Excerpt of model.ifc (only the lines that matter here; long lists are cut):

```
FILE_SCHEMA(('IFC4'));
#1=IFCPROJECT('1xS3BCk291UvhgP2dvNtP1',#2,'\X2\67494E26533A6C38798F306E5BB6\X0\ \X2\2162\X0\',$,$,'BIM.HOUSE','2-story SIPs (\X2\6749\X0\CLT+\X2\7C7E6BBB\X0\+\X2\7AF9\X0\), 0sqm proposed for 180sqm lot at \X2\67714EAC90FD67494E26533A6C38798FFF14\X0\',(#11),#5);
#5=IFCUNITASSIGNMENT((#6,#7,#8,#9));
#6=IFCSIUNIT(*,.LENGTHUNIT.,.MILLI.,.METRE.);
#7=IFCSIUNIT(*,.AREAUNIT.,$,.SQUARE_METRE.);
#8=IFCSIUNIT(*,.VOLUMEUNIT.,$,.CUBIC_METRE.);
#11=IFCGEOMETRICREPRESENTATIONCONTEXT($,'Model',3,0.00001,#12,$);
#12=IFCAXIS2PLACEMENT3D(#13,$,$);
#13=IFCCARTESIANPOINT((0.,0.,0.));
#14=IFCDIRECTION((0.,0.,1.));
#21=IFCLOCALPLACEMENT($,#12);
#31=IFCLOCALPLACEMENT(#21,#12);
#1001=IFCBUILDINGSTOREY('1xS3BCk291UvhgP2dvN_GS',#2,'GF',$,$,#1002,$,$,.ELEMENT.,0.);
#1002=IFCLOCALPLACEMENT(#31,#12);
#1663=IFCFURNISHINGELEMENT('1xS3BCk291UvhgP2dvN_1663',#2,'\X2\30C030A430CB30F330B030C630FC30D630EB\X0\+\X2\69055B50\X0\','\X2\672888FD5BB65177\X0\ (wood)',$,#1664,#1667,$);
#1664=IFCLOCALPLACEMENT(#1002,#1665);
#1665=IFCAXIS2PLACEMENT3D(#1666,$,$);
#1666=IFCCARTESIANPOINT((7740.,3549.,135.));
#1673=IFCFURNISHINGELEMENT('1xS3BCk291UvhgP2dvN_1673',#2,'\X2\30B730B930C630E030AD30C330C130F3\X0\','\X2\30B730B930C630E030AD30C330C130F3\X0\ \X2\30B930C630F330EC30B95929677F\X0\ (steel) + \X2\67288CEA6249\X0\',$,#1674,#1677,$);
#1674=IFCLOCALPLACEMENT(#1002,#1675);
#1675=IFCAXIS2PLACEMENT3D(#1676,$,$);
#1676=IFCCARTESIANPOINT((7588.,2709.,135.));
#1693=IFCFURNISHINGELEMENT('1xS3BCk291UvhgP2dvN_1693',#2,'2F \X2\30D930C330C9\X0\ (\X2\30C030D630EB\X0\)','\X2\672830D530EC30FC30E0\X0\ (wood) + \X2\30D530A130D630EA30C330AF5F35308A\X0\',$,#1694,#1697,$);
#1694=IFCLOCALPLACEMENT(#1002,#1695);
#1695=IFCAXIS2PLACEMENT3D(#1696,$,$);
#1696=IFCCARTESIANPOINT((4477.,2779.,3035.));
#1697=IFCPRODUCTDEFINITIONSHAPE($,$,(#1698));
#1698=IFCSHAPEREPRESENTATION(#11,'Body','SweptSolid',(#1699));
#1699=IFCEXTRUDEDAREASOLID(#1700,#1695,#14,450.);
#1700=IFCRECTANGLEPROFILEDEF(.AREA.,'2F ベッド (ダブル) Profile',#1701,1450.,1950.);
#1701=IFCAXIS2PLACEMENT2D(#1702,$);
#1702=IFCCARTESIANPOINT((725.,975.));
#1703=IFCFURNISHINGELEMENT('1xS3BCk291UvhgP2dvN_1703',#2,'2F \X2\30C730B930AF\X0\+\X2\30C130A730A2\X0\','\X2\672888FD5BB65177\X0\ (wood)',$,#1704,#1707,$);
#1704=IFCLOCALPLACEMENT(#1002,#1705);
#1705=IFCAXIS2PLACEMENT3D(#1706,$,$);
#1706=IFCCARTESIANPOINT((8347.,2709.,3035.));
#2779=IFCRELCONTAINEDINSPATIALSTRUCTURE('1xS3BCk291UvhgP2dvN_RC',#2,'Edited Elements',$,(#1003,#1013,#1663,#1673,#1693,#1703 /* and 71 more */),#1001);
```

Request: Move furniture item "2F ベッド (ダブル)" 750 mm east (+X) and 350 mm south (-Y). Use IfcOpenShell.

```python
import ifcopenshell
import ifcopenshell.api.geometry
import ifcopenshell.util.placement
import ifcopenshell.util.unit

model = ifcopenshell.open("model.ifc")
unit_scale = ifcopenshell.util.unit.calculate_unit_scale(model)

item = model.by_guid("1xS3BCk291UvhgP2dvN_1693")
matrix = ifcopenshell.util.placement.get_local_placement(item.ObjectPlacement)
matrix[0, 3] += 0.75 / unit_scale
matrix[1, 3] -= 0.35 / unit_scale
ifcopenshell.api.geometry.edit_object_placement(model, product=item, matrix=matrix, is_si=False)

print(ifcopenshell.util.placement.get_local_placement(item.ObjectPlacement).round(3) + 0.0)

model.write("model_rev.ifc")
```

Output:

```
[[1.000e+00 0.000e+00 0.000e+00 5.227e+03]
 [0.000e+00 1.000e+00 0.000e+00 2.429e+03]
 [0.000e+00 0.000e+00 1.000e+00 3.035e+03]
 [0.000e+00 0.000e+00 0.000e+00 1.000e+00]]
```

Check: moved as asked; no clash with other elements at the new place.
